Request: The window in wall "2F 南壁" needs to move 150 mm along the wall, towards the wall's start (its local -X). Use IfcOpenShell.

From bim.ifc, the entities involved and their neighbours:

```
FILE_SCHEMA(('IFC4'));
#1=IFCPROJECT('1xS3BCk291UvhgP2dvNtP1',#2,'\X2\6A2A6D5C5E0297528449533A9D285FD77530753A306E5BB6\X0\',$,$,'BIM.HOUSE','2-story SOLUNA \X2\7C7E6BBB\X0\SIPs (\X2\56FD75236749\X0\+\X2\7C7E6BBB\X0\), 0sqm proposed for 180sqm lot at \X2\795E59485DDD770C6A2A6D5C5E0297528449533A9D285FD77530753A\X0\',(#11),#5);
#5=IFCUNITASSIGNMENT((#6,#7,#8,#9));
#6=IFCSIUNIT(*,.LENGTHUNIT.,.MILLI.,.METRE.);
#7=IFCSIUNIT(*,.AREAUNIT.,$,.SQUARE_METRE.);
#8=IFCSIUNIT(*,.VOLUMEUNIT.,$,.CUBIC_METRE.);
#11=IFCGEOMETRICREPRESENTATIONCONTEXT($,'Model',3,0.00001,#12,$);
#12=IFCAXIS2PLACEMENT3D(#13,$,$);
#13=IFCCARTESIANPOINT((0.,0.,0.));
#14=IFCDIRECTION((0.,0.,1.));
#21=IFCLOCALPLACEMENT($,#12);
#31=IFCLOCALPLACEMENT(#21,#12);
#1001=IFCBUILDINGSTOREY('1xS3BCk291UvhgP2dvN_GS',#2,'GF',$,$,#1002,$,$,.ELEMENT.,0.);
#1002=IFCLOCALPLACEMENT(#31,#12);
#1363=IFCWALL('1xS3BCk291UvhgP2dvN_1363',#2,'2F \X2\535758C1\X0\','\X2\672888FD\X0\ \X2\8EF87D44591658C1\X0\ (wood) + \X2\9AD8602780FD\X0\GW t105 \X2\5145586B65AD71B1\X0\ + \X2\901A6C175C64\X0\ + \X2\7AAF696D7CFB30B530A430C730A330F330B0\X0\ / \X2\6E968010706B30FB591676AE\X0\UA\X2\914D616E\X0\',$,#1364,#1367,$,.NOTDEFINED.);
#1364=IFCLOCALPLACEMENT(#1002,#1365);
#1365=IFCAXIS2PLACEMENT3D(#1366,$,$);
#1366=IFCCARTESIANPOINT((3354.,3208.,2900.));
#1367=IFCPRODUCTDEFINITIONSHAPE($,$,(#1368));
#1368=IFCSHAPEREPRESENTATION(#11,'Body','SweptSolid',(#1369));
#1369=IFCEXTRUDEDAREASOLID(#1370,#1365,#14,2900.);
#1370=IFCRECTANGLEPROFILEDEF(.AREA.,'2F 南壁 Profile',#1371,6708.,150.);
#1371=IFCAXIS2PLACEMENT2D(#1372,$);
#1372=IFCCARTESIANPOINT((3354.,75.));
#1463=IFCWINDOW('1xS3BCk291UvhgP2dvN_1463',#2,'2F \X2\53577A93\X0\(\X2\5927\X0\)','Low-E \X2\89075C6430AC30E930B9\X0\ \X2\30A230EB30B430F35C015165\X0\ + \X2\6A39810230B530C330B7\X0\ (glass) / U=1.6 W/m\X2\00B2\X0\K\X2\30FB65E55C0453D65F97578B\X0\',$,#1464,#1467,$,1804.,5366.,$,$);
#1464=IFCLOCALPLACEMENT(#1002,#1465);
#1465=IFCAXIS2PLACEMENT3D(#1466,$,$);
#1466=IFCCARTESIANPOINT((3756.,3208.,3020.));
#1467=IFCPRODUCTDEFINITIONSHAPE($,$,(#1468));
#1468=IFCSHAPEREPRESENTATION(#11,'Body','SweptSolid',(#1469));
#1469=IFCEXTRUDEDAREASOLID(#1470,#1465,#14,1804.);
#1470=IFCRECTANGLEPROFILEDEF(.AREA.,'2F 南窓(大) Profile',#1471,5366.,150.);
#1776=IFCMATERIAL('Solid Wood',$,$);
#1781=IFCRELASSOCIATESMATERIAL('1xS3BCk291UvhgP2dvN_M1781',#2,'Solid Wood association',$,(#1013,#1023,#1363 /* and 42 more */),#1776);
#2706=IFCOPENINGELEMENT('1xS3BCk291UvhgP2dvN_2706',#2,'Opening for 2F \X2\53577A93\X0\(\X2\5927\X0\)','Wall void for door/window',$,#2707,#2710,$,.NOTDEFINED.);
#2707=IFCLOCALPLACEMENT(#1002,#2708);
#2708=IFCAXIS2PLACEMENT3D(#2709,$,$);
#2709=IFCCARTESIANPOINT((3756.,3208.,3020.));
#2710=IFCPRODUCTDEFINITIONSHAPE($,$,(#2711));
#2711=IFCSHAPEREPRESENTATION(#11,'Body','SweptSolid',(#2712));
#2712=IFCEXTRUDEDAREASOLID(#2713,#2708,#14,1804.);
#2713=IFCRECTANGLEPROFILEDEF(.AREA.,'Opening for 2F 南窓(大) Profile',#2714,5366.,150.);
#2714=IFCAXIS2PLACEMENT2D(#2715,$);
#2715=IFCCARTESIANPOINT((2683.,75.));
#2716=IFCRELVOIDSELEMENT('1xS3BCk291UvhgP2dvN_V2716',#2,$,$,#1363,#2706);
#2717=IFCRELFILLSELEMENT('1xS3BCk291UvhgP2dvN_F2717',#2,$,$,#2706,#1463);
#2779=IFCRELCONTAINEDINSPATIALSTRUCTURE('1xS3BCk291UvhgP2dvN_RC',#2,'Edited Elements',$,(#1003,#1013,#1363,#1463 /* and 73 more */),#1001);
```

```python
import ifcopenshell
import ifcopenshell.api.geometry
import ifcopenshell.util.placement
import ifcopenshell.util.unit

model = ifcopenshell.open("bim.ifc")
unit_scale = ifcopenshell.util.unit.calculate_unit_scale(model)

window = model.by_guid("1xS3BCk291UvhgP2dvN_1463")
opening = window.FillsVoids[0].RelatingOpeningElement
wall = opening.VoidsElements[0].RelatingBuildingElement

wall_matrix = ifcopenshell.util.placement.get_local_placement(wall.ObjectPlacement)
shift = wall_matrix[:3, 0] * -0.15 / unit_scale
before = ifcopenshell.util.placement.get_local_placement(window.ObjectPlacement)[:3, 3].copy()

# The window is not placed relative to its opening, so move both.
for product in (opening, window):
    matrix = ifcopenshell.util.placement.get_local_placement(product.ObjectPlacement)
    matrix[:3, 3] += shift
    ifcopenshell.api.geometry.edit_object_placement(model, product=product, matrix=matrix, is_si=False)

after = ifcopenshell.util.placement.get_local_placement(window.ObjectPlacement)[:3, 3]
print("window moved by", (after - before).round(3) + 0.0)

model.write("bim-out.ifc")
```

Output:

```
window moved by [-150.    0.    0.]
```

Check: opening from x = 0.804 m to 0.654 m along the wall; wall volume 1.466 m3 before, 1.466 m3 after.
